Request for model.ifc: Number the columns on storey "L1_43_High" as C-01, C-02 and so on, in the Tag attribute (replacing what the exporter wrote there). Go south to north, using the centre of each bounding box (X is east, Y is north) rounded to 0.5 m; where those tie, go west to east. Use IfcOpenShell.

First a look at what the model holds.

```python
import ifcopenshell
import ifcopenshell.util.element
import ifcopenshell.util.placement

model = ifcopenshell.open("model.ifc")
print(model.schema)
storey = next(s for s in model.by_type("IfcBuildingStorey") if s.Name == "L1_43_High")
columns = [e for e in ifcopenshell.util.element.get_decomposition(storey) if e.is_a("IfcColumn")]
for e in sorted(columns, key=lambda e: e.id()):
    origin = ifcopenshell.util.placement.get_local_placement(e.ObjectPlacement)[:3, 3]
    print(e.id(), e.Tag, e.Name, origin.round(2) + 0.0, sep=" | ")
```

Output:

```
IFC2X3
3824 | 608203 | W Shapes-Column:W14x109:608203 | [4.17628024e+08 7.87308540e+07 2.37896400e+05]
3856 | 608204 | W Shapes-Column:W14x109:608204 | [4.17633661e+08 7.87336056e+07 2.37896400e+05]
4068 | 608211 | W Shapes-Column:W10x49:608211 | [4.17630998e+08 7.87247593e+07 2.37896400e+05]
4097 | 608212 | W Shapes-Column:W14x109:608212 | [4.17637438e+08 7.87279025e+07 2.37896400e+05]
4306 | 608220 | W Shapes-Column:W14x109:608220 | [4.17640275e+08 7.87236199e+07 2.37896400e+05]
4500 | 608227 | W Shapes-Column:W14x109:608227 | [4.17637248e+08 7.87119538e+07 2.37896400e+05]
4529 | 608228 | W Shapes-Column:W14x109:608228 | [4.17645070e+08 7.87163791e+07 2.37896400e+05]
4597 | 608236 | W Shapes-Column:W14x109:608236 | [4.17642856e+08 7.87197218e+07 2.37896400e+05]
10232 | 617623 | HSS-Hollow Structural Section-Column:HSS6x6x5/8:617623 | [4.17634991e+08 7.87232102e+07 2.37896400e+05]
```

```python
import ifcopenshell
import ifcopenshell.geom
import ifcopenshell.util.element
import ifcopenshell.util.shape

model = ifcopenshell.open("model.ifc")
settings = ifcopenshell.geom.settings()
settings.set("use-world-coords", True)


def centre(element):
    shape = ifcopenshell.geom.create_shape(settings, element)
    return ifcopenshell.util.shape.get_bbox_centroid(shape.geometry)


storey = next(s for s in model.by_type("IfcBuildingStorey") if s.Name == "L1_43_High")
columns = [e for e in ifcopenshell.util.element.get_decomposition(storey) if e.is_a("IfcColumn")]

# Insertion points can sit at a corner or the storey origin, so sort by the geometry (in metres).
centres = {e: centre(e) for e in columns}
columns.sort(key=lambda e: (round(centres[e][1] / 0.5), centres[e][0]))

for i, e in enumerate(columns, start=1):
    number = f"C-{i:02d}"
    e.Tag = number
    print(e.id(), number)

model.write("model-out.ifc")
```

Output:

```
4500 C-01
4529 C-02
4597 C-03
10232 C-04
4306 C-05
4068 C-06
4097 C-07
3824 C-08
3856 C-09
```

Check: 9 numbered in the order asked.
